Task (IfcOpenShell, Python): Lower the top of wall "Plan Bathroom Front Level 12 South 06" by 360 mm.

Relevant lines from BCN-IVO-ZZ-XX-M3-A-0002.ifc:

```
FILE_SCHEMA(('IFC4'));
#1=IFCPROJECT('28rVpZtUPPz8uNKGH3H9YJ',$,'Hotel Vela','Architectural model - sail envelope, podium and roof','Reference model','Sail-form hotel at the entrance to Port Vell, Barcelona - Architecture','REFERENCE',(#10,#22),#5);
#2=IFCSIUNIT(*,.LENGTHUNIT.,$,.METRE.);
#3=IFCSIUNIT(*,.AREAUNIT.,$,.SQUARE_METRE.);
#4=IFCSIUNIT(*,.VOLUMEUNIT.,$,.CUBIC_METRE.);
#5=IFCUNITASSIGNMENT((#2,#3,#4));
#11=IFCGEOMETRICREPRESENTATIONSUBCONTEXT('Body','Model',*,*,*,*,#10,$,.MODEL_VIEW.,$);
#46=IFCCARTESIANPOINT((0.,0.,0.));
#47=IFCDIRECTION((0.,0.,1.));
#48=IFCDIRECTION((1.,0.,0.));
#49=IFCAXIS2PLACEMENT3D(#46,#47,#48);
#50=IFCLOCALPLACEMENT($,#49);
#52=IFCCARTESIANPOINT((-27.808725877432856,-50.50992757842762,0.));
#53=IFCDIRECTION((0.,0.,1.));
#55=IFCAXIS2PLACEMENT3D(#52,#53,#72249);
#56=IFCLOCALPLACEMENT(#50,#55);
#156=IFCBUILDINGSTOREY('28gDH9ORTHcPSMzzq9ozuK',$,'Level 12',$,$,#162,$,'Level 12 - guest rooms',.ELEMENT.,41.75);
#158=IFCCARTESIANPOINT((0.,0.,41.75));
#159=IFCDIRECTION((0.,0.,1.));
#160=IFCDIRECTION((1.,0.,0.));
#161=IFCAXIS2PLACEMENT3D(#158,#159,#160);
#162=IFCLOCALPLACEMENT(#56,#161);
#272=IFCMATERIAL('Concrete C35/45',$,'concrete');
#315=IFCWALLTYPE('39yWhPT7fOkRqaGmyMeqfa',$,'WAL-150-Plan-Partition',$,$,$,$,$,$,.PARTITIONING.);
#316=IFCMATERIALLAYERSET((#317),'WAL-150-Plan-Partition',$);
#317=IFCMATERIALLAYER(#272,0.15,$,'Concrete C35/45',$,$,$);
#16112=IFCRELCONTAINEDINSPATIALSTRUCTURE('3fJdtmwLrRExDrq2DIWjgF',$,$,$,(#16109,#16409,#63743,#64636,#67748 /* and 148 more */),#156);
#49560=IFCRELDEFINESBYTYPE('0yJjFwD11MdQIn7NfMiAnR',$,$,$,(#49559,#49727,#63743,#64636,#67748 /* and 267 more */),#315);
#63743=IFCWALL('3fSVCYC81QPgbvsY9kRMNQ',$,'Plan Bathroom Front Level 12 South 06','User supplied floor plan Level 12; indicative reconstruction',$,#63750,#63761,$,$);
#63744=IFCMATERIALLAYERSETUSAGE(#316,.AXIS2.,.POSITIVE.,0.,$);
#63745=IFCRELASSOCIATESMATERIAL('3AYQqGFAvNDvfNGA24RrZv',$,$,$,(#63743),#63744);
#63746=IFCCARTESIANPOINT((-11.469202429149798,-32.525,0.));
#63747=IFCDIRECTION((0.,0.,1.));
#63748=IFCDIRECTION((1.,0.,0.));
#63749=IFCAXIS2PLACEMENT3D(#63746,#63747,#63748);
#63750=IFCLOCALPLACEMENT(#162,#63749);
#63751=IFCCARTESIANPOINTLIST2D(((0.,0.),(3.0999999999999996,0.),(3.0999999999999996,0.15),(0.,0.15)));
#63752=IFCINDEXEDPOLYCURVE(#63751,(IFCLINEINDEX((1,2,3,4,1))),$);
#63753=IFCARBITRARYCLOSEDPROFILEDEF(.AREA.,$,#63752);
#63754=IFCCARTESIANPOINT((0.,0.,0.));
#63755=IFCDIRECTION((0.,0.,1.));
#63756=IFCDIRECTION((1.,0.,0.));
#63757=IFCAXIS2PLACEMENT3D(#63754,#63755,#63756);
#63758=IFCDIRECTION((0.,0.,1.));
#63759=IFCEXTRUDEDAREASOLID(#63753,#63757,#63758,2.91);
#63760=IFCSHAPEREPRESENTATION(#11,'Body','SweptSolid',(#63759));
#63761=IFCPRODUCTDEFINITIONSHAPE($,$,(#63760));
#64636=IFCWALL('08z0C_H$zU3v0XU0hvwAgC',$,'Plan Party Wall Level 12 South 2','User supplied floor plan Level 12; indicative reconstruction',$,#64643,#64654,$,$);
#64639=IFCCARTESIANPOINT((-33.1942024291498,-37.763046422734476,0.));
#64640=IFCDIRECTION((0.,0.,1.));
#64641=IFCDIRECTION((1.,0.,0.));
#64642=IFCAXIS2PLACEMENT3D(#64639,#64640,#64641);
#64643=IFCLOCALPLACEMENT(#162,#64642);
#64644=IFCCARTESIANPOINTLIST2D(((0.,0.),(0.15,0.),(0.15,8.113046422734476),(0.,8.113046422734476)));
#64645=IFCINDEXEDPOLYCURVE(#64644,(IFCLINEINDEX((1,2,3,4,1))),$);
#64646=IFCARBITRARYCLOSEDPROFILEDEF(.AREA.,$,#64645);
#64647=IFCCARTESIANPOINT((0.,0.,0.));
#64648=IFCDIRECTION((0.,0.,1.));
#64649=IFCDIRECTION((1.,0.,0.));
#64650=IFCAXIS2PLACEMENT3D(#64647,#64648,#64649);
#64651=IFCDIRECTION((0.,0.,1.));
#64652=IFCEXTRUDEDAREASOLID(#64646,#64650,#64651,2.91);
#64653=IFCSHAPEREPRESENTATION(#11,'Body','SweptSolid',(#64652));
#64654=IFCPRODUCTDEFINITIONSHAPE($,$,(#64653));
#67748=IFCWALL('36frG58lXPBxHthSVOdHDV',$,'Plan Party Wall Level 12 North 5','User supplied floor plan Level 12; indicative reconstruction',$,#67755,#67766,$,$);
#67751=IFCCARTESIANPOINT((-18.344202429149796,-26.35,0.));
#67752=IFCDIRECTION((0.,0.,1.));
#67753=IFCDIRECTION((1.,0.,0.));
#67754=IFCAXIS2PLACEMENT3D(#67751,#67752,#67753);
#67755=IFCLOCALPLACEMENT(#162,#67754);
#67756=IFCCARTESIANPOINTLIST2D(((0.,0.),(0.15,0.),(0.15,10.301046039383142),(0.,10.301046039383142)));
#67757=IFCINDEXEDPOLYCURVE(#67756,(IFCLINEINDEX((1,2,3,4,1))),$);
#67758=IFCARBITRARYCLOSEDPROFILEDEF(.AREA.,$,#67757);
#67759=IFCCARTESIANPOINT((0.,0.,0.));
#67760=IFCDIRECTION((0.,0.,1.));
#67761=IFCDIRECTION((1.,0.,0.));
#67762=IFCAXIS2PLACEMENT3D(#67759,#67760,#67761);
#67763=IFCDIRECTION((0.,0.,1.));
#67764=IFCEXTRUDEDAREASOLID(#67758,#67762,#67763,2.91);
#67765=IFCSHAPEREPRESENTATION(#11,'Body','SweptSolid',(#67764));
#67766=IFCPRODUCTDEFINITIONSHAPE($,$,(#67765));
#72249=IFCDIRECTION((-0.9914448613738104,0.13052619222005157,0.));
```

```python
import ifcopenshell
import ifcopenshell.geom
import ifcopenshell.util.representation
import ifcopenshell.util.shape
import ifcopenshell.util.unit

model = ifcopenshell.open("BCN-IVO-ZZ-XX-M3-A-0002.ifc")
unit_scale = ifcopenshell.util.unit.calculate_unit_scale(model)
settings = ifcopenshell.geom.settings()


def volume(element):
    """Net volume in cubic metres, openings subtracted."""
    shape = ifcopenshell.geom.create_shape(settings, element)
    return ifcopenshell.util.shape.get_volume(shape.geometry)


wall = model.by_guid("3fSVCYC81QPgbvsY9kRMNQ")
before = volume(wall)

body = ifcopenshell.util.representation.get_representation(wall, "Model", "Body")
solid = body.Items[0]
old_height = solid.Depth
solid.Depth -= 0.36 / unit_scale
after = volume(wall)

print(f"height {old_height:g} -> {solid.Depth:g}, volume {before:.3f} -> {after:.3f} m3")

model.write("BCN-IVO-ZZ-XX-M3-A-0002-out.ifc")
```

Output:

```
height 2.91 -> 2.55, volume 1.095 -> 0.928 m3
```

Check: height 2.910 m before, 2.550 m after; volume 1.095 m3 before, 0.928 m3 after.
